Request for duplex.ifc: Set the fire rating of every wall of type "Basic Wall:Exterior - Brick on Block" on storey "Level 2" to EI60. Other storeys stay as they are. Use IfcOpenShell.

First a look at what the model holds.

```python
import ifcopenshell
import ifcopenshell.util.element

model = ifcopenshell.open("duplex.ifc")
print(model.schema)
storey = next(s for s in model.by_type("IfcBuildingStorey") if s.Name == "Level 2")
walls = [e for e in ifcopenshell.util.element.get_decomposition(storey) if e.is_a("IfcWall")]
seen = {}
for e in walls:
    element_type = ifcopenshell.util.element.get_type(e)
    key = (element_type.Name if element_type != e and element_type else None, ifcopenshell.util.element.get_pset(e, "Pset_WallCommon", "FireRating"))
    seen[key] = seen.get(key, 0) + 1
for (name, value), count in sorted(seen.items(), key=str):
    print(count, "x", name, "|", value)
```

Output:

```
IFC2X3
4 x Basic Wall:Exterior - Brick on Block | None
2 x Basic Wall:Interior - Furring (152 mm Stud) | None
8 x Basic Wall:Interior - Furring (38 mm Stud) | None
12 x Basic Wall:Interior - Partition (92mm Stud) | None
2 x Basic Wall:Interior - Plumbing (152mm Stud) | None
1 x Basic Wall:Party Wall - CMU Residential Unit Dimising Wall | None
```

```python
import ifcopenshell
import ifcopenshell.api.pset
import ifcopenshell.util.element

model = ifcopenshell.open("duplex.ifc")

storey = next(s for s in model.by_type("IfcBuildingStorey") if s.Name == "Level 2")
walls = [e for e in ifcopenshell.util.element.get_decomposition(storey) if e.is_a("IfcWall")]

count = 0
for e in walls:
    element_type = ifcopenshell.util.element.get_type(e)
    if element_type in (None, e) or element_type.Name != "Basic Wall:Exterior - Brick on Block":
        continue
    # add_pset returns the element's existing set when there is one.
    pset = ifcopenshell.api.pset.add_pset(model, product=e, name="Pset_WallCommon")
    ifcopenshell.api.pset.edit_pset(model, pset=pset, properties={"FireRating": "EI60"})
    count += 1

print(count, "walls updated")

model.write("duplex_v2.ifc")
```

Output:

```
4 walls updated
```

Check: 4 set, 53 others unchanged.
